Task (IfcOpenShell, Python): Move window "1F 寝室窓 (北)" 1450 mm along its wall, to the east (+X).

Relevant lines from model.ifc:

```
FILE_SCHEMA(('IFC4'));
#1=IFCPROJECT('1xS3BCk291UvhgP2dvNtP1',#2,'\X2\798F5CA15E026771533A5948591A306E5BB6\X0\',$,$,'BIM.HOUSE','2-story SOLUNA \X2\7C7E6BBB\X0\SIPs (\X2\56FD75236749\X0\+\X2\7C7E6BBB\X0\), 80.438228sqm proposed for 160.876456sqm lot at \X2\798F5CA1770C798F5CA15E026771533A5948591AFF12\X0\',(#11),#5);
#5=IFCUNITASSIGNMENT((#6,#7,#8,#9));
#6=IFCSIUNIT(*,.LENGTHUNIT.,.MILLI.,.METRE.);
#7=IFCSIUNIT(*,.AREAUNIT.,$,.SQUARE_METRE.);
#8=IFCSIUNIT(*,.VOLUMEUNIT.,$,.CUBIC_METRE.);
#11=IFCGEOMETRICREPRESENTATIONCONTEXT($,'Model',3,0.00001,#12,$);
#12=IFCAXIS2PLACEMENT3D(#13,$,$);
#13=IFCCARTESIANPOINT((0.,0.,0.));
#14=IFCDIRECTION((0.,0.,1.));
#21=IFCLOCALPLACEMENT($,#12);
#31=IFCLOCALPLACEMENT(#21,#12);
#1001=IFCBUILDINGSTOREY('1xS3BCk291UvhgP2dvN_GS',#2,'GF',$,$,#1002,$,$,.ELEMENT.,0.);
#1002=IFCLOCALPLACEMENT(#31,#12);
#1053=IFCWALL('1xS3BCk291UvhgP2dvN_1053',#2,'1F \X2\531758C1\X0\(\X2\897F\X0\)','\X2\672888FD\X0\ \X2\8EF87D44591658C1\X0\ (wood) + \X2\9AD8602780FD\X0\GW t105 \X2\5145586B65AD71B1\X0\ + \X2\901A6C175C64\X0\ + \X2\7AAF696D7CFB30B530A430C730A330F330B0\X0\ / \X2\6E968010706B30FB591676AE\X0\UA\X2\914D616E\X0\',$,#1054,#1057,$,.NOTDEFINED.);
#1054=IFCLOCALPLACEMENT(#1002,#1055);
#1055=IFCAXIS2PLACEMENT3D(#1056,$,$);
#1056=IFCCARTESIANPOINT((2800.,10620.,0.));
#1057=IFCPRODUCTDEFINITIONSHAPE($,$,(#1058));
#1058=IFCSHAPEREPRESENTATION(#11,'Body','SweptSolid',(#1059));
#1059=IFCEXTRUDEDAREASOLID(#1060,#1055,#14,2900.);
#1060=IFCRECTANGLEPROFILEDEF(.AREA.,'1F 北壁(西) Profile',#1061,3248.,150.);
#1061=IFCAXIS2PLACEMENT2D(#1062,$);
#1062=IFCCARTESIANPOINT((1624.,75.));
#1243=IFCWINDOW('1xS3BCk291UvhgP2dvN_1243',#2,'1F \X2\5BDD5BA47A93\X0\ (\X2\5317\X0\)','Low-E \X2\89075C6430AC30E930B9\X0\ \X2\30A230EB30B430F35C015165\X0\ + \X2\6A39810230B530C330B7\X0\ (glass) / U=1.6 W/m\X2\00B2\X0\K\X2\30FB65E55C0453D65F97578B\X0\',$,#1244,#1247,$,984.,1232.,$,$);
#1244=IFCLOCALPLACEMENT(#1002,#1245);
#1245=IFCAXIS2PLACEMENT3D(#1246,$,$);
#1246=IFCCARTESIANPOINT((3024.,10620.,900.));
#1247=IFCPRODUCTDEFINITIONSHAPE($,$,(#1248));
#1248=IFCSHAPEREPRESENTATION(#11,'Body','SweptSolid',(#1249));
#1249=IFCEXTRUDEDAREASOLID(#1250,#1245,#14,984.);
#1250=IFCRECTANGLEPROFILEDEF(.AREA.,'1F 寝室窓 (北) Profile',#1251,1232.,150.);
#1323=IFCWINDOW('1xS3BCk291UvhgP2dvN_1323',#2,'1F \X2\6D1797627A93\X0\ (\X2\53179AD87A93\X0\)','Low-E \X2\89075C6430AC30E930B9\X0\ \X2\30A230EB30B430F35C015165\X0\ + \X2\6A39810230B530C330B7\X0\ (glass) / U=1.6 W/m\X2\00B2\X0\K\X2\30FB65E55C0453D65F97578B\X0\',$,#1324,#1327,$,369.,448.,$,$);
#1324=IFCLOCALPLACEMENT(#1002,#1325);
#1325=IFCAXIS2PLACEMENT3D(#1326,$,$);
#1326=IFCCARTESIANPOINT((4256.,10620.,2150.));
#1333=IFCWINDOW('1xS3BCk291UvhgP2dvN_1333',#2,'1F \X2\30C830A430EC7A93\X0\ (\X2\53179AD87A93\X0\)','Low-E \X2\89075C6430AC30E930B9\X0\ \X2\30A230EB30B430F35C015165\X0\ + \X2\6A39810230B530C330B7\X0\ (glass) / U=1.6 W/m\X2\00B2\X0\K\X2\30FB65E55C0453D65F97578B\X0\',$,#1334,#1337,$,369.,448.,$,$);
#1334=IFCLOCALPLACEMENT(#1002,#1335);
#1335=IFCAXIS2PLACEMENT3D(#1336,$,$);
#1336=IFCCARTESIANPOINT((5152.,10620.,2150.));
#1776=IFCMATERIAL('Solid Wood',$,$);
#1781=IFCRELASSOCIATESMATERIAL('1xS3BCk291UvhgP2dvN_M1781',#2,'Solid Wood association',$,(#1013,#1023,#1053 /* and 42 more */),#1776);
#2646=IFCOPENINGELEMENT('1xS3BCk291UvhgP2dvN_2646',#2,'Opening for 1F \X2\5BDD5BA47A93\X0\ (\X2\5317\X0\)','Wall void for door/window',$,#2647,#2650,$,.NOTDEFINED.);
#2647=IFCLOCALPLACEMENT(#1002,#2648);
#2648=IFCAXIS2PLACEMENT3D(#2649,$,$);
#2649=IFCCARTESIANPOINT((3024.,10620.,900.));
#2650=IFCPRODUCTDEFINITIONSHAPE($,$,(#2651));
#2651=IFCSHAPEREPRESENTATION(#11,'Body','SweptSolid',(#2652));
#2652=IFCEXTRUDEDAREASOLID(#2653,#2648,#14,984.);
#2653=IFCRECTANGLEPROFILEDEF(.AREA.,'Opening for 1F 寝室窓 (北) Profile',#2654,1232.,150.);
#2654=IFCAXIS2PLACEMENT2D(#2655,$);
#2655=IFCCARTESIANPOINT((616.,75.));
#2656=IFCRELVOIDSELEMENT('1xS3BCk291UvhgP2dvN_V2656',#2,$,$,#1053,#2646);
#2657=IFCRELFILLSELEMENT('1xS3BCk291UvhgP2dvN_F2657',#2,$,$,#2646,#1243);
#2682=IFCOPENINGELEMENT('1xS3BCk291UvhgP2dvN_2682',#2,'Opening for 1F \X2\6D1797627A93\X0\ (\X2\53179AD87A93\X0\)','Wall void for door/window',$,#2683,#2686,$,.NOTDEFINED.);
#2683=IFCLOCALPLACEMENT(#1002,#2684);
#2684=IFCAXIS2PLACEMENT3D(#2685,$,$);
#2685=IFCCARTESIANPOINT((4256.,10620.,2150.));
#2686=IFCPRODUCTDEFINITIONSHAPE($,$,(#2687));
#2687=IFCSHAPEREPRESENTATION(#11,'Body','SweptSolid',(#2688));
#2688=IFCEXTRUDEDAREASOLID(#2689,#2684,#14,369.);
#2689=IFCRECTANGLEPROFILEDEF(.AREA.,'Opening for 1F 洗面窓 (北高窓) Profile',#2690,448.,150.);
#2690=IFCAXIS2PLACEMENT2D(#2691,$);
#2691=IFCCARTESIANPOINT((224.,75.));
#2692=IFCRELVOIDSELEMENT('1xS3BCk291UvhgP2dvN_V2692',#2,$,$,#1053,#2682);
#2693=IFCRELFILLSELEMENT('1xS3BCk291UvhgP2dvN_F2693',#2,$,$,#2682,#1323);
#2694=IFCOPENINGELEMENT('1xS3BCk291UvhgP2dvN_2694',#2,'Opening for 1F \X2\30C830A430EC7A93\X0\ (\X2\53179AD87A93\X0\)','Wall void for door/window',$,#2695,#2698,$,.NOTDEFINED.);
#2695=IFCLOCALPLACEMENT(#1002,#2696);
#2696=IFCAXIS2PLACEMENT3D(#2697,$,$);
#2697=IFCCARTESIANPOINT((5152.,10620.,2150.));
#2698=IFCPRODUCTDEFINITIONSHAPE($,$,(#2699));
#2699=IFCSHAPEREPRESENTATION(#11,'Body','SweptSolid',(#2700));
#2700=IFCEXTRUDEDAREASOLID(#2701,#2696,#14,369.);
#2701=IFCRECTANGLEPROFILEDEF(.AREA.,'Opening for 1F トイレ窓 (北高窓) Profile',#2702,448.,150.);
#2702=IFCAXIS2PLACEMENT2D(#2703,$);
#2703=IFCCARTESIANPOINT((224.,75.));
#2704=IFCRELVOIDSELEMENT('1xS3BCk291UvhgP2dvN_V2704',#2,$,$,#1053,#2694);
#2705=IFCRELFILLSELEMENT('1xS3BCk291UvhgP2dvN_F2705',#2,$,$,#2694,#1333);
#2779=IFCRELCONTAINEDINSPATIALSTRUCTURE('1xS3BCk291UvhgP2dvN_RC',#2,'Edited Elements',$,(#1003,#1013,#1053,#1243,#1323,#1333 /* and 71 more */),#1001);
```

```python
import ifcopenshell
import ifcopenshell.api.geometry
import ifcopenshell.util.placement
import ifcopenshell.util.unit

model = ifcopenshell.open("model.ifc")
unit_scale = ifcopenshell.util.unit.calculate_unit_scale(model)

window = model.by_guid("1xS3BCk291UvhgP2dvN_1243")
opening = window.FillsVoids[0].RelatingOpeningElement
wall = opening.VoidsElements[0].RelatingBuildingElement

wall_matrix = ifcopenshell.util.placement.get_local_placement(wall.ObjectPlacement)
shift = wall_matrix[:3, 0] * 1.45 / unit_scale
before = ifcopenshell.util.placement.get_local_placement(window.ObjectPlacement)[:3, 3].copy()

# The window is not placed relative to its opening, so move both.
for product in (opening, window):
    matrix = ifcopenshell.util.placement.get_local_placement(product.ObjectPlacement)
    matrix[:3, 3] += shift
    ifcopenshell.api.geometry.edit_object_placement(model, product=product, matrix=matrix, is_si=False)

after = ifcopenshell.util.placement.get_local_placement(window.ObjectPlacement)[:3, 3]
print("window moved by", (after - before).round(3) + 0.0)

model.write("model_v2.ifc")
```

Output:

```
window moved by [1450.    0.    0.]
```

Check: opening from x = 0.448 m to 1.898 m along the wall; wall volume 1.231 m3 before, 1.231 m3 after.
